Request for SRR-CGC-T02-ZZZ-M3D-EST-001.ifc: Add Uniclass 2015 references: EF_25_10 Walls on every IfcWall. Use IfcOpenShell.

First a look at what the model holds.

```python
import ifcopenshell

model = ifcopenshell.open("SRR-CGC-T02-ZZZ-M3D-EST-001.ifc")
print(model.schema)
print("classifications:", [c.Name for c in model.by_type("IfcClassification")])
for ifc_class in ("IfcDoor", "IfcRoof", "IfcStair", "IfcWall", "IfcWindow"):
    print(ifc_class, len(model.by_type(ifc_class)))
```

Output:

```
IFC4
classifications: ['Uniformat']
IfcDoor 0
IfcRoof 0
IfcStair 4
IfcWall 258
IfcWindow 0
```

```python
import ifcopenshell
import ifcopenshell.api.classification

model = ifcopenshell.open("SRR-CGC-T02-ZZZ-M3D-EST-001.ifc")

system = ifcopenshell.api.classification.add_classification(model, classification="Uniclass 2015")

codes = {
    "IfcWall": ("EF_25_10", "Walls"),
}
for ifc_class, (code, name) in codes.items():
    products = model.by_type(ifc_class)
    ifcopenshell.api.classification.add_reference(
        model, products=products, classification=system, identification=code, name=name
    )
    print(code, len(products))

model.write("SRR-CGC-T02-ZZZ-M3D-EST-001_edited.ifc")
```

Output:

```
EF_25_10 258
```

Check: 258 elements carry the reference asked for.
